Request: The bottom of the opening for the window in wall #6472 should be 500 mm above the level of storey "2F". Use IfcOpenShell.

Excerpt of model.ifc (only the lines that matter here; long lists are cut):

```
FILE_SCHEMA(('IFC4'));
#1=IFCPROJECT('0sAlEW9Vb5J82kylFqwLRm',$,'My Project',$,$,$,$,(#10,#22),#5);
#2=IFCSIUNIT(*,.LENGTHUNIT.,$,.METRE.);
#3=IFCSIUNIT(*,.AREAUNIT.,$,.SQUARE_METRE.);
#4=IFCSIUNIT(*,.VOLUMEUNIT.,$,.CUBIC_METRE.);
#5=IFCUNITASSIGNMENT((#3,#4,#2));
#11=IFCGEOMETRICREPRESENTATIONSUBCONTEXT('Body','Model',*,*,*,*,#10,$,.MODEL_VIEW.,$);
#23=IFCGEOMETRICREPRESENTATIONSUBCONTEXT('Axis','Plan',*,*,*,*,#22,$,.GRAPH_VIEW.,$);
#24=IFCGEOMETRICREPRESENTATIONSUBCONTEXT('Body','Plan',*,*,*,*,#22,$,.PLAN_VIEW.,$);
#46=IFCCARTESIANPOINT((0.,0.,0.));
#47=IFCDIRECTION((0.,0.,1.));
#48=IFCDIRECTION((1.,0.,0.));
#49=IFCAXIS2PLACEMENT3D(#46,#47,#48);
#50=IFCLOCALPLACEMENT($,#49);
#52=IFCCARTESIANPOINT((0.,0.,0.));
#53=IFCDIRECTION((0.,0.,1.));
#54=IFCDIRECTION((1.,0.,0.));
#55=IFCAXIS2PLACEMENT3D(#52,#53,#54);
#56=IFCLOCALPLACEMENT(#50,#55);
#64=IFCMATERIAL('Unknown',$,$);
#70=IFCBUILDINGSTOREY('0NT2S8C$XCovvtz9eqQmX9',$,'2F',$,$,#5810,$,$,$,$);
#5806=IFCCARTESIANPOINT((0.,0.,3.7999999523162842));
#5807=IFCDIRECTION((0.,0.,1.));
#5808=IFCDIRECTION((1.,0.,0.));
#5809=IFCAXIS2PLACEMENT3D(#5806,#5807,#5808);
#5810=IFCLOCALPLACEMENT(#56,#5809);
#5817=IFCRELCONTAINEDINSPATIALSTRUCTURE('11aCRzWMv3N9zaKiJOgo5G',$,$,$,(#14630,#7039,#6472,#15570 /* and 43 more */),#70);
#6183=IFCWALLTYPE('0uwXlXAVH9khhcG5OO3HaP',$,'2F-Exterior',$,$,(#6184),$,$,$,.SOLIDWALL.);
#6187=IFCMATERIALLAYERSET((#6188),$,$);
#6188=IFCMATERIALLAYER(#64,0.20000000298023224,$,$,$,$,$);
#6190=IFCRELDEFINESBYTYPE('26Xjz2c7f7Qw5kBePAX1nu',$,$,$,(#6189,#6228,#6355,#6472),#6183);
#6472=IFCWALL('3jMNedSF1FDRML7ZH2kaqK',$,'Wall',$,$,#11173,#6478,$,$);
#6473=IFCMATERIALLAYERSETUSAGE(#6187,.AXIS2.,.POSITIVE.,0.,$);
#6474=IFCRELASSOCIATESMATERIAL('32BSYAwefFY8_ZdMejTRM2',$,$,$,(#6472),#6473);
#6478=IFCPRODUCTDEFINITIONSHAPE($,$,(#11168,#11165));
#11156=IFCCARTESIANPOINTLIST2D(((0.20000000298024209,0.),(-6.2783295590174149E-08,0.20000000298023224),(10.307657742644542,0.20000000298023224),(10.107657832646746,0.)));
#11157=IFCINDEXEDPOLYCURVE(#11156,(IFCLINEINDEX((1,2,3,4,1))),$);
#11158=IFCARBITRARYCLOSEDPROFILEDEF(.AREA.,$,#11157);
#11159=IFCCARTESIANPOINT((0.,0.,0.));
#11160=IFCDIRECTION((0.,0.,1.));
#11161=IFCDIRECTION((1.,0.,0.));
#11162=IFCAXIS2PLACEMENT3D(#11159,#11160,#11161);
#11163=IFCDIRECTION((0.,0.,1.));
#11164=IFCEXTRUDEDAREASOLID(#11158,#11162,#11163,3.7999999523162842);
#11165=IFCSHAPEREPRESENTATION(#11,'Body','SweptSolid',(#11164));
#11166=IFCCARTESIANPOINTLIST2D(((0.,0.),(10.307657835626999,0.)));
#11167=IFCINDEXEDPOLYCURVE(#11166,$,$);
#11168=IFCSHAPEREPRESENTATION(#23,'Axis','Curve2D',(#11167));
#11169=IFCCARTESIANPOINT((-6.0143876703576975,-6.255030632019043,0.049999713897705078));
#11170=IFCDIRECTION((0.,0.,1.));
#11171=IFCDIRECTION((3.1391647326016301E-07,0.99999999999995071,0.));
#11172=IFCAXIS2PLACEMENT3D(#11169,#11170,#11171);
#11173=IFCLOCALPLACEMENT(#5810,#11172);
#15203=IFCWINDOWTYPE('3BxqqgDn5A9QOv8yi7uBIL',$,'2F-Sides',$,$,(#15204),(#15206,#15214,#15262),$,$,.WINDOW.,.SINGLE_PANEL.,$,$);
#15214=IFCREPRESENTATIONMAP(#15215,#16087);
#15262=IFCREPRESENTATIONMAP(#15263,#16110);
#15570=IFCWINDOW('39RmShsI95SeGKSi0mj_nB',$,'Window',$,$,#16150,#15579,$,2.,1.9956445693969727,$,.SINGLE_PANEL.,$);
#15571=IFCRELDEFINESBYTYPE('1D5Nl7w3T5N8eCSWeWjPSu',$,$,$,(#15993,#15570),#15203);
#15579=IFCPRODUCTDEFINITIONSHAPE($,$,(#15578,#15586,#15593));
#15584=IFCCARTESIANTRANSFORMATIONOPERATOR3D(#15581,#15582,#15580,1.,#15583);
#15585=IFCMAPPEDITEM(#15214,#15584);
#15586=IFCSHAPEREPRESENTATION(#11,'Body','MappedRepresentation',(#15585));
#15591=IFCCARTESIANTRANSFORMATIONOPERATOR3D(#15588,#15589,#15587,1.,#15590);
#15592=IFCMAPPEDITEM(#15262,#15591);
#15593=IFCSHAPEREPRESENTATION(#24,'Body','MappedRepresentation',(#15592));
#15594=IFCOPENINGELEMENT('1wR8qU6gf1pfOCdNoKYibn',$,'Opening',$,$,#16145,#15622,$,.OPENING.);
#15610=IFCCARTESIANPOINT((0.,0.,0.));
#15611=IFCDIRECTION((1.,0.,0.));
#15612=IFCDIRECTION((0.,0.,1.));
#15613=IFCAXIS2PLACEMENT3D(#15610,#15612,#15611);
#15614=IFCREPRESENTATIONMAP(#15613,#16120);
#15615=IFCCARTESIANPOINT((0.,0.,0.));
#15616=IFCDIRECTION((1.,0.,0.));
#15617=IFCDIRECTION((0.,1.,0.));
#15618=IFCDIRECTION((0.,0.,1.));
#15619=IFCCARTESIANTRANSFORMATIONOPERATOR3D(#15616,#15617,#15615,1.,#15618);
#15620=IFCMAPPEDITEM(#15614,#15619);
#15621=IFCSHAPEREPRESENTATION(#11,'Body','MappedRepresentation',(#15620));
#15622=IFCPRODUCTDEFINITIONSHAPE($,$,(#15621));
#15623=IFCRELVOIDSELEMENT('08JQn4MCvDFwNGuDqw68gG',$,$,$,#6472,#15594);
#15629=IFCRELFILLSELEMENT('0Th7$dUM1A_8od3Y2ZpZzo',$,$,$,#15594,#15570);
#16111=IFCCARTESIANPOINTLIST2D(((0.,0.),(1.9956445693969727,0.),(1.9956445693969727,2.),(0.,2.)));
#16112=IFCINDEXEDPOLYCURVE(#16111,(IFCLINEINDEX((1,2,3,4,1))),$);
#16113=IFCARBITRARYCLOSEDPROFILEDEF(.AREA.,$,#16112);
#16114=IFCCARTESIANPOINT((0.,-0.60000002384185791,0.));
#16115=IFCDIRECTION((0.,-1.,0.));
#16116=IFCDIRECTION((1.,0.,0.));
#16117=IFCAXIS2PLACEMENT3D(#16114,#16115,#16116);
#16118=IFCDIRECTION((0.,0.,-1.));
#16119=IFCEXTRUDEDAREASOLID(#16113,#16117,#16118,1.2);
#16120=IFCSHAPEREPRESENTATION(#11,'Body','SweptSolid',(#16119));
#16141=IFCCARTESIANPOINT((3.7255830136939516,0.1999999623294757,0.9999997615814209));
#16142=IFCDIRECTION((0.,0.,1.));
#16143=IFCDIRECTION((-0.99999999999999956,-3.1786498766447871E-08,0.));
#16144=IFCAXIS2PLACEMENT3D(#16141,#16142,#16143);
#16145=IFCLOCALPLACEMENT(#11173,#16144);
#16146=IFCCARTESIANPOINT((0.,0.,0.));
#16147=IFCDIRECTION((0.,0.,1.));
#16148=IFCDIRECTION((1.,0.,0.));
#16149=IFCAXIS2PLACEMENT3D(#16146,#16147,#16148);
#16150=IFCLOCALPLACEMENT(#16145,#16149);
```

```python
import numpy as np
import ifcopenshell
import ifcopenshell.api.geometry
import ifcopenshell.geom
import ifcopenshell.util.element
import ifcopenshell.util.placement
import ifcopenshell.util.shape
import ifcopenshell.util.unit

model = ifcopenshell.open("model.ifc")
unit_scale = ifcopenshell.util.unit.calculate_unit_scale(model)

window = model.by_guid("39RmShsI95SeGKSi0mj_nB")
opening = window.FillsVoids[0].RelatingOpeningElement
storey = ifcopenshell.util.element.get_container(window, ifc_class="IfcBuildingStorey")
level = ifcopenshell.util.placement.get_local_placement(storey.ObjectPlacement)[2, 3]

# The opening's origin need not be at the sill, so measure its lowest point.
shape = ifcopenshell.geom.create_shape(ifcopenshell.geom.settings(), opening)
bottom = ifcopenshell.util.shape.get_shape_bottom_elevation(shape, shape.geometry) / unit_scale
dz = level + 0.5 / unit_scale - bottom

shift = np.array([0.0, 0.0, dz])
# The window is placed relative to its opening, so it follows when the opening moves.
matrix = ifcopenshell.util.placement.get_local_placement(opening.ObjectPlacement)
matrix[:3, 3] += shift
ifcopenshell.api.geometry.edit_object_placement(
    model, product=opening, matrix=matrix, is_si=False, should_transform_children=True
)

print(f"moved by {dz * unit_scale:+.3f} m")

model.write("model-out.ifc")
```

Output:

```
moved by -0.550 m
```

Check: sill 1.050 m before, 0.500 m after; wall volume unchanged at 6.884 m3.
